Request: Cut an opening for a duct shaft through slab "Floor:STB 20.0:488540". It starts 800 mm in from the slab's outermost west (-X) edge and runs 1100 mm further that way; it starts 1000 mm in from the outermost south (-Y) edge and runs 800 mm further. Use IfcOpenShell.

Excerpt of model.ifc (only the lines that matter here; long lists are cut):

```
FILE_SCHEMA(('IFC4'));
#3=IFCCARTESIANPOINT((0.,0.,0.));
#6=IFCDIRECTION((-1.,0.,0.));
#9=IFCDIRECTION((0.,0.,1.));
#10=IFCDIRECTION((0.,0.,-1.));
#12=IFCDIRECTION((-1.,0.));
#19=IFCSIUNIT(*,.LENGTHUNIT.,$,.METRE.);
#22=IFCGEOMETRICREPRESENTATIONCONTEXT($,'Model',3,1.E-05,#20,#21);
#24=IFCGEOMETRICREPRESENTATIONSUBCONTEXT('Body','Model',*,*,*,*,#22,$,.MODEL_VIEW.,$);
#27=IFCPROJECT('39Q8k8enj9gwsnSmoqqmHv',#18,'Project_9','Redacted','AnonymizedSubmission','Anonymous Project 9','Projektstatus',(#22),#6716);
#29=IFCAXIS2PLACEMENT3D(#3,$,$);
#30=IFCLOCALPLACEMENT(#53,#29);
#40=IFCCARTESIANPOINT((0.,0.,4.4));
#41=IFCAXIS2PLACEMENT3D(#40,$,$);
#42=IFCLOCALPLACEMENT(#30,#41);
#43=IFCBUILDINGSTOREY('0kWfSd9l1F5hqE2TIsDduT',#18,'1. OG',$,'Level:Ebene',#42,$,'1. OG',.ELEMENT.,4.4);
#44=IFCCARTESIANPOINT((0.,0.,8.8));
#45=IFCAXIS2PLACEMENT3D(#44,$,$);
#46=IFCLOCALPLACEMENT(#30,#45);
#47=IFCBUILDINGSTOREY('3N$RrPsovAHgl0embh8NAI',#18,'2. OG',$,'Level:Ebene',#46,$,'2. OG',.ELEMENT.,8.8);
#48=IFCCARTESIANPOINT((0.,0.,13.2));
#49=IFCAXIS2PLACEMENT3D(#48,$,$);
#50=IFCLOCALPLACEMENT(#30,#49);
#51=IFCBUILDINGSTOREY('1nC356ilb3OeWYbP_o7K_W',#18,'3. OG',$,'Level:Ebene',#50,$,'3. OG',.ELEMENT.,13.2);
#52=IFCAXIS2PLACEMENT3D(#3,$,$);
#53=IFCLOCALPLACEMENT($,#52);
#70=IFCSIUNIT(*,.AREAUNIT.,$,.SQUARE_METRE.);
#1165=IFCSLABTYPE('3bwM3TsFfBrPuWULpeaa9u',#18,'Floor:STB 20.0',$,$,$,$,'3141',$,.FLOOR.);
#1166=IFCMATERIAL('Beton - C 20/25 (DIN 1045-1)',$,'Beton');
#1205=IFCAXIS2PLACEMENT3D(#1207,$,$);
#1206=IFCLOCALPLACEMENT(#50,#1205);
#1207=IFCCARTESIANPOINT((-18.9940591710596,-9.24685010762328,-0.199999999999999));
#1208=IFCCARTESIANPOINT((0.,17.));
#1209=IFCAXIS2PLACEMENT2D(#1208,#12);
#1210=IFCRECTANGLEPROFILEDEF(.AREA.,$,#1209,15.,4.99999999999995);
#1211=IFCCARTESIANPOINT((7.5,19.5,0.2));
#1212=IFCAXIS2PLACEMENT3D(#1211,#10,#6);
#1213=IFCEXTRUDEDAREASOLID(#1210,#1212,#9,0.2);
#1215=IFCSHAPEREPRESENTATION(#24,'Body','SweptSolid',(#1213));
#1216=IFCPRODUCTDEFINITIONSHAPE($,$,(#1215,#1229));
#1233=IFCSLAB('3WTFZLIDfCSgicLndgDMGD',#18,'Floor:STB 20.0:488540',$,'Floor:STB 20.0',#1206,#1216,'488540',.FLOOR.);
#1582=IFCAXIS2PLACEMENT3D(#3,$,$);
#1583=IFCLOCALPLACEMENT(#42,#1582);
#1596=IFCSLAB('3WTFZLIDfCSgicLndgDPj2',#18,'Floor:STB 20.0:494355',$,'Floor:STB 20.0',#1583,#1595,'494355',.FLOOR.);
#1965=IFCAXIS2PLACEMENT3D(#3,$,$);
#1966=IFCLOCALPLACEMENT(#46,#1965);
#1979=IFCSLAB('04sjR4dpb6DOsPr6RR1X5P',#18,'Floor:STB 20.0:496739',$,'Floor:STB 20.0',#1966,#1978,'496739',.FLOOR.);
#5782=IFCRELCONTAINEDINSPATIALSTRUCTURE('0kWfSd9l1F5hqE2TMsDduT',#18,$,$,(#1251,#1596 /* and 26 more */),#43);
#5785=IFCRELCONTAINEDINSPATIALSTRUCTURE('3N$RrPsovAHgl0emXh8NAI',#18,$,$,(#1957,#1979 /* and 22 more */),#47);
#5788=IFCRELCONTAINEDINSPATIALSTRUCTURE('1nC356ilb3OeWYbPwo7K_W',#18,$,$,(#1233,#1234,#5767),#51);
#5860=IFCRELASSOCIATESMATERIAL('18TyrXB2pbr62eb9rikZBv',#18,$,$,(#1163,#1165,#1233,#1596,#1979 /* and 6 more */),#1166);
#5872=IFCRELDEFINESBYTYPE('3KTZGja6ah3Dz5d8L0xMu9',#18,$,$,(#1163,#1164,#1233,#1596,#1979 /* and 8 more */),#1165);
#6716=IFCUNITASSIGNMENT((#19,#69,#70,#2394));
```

```python
import numpy as np
import ifcopenshell
import ifcopenshell.api.feature
import ifcopenshell.api.geometry
import ifcopenshell.api.root
import ifcopenshell.geom
import ifcopenshell.util.placement
import ifcopenshell.util.representation
import ifcopenshell.util.shape
import ifcopenshell.util.unit

model = ifcopenshell.open("model.ifc")
unit_scale = ifcopenshell.util.unit.calculate_unit_scale(model)
settings = ifcopenshell.geom.settings()


def volume(element):
    """Net volume in cubic metres, openings subtracted."""
    shape = ifcopenshell.geom.create_shape(settings, element)
    return ifcopenshell.util.shape.get_volume(shape.geometry)


slab = model.by_guid("3WTFZLIDfCSgicLndgDMGD")
before = volume(slab)

# Extent in the slab's own axes, in metres. The edges named are its -X and -Y sides.
slab_shape = ifcopenshell.geom.create_shape(settings, slab)
vertices = ifcopenshell.util.shape.get_vertices(slab_shape.geometry)
x_min, y_min, bottom = vertices.min(axis=0)
top = vertices[:, 2].max()

opening = ifcopenshell.api.root.create_entity(model, ifc_class="IfcOpeningElement", name="Duct shaft opening", predefined_type="OPENING")
context = ifcopenshell.util.representation.get_context(model, "Model", "Body", "MODEL_VIEW")
width, depth = 1.1, 0.8
outline = [(0.0, 0.0), (width, 0.0), (width, depth), (0.0, depth), (0.0, 0.0)]
# Overshoot both faces by 50 mm so the cut is clean.
shape = ifcopenshell.api.geometry.add_slab_representation(
    model, context=context, depth=top - bottom + 0.1, polyline=outline
)
ifcopenshell.api.geometry.assign_representation(model, product=opening, representation=shape)

matrix = ifcopenshell.util.placement.get_local_placement(slab.ObjectPlacement)
matrix[:, 3] = matrix @ np.append(np.array([x_min + 0.8, y_min + 1, bottom - 0.05]) / unit_scale, 1.0)
ifcopenshell.api.geometry.edit_object_placement(model, product=opening, matrix=matrix, is_si=False)
ifcopenshell.api.feature.add_feature(model, feature=opening, element=slab)

after = volume(slab)

print(f"slab volume {before:.3f} -> {after:.3f} m3")

model.write("model_rev.ifc")
```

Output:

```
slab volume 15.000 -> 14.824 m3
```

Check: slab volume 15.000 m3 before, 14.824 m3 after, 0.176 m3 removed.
